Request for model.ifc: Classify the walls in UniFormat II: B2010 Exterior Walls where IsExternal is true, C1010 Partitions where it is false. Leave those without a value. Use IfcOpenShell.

First a look at what the model holds.

```python
import ifcopenshell
import ifcopenshell.util.element

model = ifcopenshell.open("model.ifc")
print(model.schema)
print("classifications:", [c.Name for c in model.by_type("IfcClassification")])
values = [ifcopenshell.util.element.get_pset(e, "Pset_WallCommon", "IsExternal") for e in model.by_type("IfcWall")]
for value in (True, False, None):
    print("IsExternal", value, values.count(value))
```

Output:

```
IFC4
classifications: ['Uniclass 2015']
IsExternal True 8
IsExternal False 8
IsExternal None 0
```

```python
import ifcopenshell
import ifcopenshell.api.classification
import ifcopenshell.util.element

model = ifcopenshell.open("model.ifc")

system = ifcopenshell.api.classification.add_classification(model, classification="UniFormat II")

walls = model.by_type("IfcWall")
external = {e: ifcopenshell.util.element.get_pset(e, "Pset_WallCommon", "IsExternal") for e in walls}
for flag, code, name in ((True, "B2010", "Exterior Walls"), (False, "C1010", "Partitions")):
    products = [e for e in walls if external[e] is flag]
    ifcopenshell.api.classification.add_reference(
        model, products=products, classification=system, identification=code, name=name
    )
    print(code, len(products))

model.write("model_v2.ifc")
```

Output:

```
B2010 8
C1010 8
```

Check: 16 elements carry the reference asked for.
